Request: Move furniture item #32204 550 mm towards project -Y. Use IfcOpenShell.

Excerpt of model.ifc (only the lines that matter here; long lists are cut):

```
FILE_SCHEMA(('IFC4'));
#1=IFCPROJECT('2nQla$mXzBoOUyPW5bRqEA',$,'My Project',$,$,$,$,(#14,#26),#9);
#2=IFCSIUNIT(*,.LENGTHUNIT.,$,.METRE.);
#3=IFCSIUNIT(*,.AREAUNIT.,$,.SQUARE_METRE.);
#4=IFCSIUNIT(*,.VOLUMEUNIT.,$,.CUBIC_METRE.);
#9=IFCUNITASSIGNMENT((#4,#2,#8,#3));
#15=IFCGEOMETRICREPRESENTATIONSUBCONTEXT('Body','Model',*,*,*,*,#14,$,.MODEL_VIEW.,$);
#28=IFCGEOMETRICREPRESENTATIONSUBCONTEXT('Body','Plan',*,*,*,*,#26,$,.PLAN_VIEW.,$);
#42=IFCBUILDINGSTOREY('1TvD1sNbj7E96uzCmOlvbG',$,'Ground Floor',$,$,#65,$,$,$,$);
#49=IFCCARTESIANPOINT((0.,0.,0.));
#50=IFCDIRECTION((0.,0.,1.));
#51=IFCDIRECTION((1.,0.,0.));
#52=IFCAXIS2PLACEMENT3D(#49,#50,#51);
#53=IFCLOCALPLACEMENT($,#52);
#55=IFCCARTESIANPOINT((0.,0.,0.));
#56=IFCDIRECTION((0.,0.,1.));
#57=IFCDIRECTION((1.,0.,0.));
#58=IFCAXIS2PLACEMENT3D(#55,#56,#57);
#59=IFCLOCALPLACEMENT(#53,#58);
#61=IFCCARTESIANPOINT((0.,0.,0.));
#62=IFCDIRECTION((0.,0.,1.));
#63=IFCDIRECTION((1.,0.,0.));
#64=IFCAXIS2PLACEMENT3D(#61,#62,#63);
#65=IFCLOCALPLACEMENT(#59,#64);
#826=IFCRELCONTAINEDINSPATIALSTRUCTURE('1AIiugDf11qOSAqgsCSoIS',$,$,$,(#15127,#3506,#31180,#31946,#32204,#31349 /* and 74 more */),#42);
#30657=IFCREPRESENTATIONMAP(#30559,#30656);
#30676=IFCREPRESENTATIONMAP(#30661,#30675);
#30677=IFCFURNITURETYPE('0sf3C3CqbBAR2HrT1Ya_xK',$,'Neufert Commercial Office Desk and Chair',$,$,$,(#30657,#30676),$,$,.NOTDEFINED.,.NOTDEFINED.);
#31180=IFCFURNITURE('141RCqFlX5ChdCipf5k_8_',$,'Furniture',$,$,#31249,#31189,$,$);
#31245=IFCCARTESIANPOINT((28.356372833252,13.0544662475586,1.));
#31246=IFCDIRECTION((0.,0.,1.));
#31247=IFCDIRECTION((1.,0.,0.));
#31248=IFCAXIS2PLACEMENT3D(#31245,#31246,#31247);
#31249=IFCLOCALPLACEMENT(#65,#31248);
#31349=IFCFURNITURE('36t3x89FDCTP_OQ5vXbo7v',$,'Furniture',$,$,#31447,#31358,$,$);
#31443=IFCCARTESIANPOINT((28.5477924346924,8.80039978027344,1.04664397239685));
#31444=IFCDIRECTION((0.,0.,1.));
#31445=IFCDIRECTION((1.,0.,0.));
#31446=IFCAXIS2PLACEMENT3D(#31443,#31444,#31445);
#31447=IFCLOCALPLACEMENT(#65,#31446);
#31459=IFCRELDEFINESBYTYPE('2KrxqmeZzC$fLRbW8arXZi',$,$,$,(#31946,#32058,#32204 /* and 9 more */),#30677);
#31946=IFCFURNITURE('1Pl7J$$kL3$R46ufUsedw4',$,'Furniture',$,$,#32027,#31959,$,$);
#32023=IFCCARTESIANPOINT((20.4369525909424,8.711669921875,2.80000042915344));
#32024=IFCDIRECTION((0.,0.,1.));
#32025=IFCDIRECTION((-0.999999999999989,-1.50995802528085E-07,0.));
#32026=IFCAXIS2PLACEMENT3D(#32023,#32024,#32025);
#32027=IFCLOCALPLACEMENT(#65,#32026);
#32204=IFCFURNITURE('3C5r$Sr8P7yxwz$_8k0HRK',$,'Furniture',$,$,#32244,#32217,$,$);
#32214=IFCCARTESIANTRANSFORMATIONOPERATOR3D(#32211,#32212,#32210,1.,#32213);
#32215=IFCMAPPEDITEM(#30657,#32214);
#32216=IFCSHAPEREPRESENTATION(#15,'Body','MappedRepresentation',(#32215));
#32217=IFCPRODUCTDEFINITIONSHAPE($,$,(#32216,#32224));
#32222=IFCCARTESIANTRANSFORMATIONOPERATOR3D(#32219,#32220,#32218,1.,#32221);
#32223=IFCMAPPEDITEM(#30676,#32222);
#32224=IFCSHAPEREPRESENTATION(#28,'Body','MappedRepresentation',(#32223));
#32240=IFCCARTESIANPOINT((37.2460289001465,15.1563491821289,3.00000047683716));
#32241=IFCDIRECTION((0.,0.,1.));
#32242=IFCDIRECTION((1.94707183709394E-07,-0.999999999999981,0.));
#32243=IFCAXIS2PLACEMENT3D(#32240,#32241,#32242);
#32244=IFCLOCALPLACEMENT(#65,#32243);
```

```python
import ifcopenshell
import ifcopenshell.api.geometry
import ifcopenshell.util.placement

model = ifcopenshell.open("model.ifc")

item = model.by_guid("3C5r$Sr8P7yxwz$_8k0HRK")
matrix = ifcopenshell.util.placement.get_local_placement(item.ObjectPlacement)
matrix[1, 3] -= 0.55
ifcopenshell.api.geometry.edit_object_placement(model, product=item, matrix=matrix, is_si=False)

print(ifcopenshell.util.placement.get_local_placement(item.ObjectPlacement).round(3) + 0.0)

model.write("model_rev.ifc")
```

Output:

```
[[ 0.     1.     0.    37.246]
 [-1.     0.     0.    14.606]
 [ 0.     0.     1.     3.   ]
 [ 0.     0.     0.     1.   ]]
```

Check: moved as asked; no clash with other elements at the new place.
